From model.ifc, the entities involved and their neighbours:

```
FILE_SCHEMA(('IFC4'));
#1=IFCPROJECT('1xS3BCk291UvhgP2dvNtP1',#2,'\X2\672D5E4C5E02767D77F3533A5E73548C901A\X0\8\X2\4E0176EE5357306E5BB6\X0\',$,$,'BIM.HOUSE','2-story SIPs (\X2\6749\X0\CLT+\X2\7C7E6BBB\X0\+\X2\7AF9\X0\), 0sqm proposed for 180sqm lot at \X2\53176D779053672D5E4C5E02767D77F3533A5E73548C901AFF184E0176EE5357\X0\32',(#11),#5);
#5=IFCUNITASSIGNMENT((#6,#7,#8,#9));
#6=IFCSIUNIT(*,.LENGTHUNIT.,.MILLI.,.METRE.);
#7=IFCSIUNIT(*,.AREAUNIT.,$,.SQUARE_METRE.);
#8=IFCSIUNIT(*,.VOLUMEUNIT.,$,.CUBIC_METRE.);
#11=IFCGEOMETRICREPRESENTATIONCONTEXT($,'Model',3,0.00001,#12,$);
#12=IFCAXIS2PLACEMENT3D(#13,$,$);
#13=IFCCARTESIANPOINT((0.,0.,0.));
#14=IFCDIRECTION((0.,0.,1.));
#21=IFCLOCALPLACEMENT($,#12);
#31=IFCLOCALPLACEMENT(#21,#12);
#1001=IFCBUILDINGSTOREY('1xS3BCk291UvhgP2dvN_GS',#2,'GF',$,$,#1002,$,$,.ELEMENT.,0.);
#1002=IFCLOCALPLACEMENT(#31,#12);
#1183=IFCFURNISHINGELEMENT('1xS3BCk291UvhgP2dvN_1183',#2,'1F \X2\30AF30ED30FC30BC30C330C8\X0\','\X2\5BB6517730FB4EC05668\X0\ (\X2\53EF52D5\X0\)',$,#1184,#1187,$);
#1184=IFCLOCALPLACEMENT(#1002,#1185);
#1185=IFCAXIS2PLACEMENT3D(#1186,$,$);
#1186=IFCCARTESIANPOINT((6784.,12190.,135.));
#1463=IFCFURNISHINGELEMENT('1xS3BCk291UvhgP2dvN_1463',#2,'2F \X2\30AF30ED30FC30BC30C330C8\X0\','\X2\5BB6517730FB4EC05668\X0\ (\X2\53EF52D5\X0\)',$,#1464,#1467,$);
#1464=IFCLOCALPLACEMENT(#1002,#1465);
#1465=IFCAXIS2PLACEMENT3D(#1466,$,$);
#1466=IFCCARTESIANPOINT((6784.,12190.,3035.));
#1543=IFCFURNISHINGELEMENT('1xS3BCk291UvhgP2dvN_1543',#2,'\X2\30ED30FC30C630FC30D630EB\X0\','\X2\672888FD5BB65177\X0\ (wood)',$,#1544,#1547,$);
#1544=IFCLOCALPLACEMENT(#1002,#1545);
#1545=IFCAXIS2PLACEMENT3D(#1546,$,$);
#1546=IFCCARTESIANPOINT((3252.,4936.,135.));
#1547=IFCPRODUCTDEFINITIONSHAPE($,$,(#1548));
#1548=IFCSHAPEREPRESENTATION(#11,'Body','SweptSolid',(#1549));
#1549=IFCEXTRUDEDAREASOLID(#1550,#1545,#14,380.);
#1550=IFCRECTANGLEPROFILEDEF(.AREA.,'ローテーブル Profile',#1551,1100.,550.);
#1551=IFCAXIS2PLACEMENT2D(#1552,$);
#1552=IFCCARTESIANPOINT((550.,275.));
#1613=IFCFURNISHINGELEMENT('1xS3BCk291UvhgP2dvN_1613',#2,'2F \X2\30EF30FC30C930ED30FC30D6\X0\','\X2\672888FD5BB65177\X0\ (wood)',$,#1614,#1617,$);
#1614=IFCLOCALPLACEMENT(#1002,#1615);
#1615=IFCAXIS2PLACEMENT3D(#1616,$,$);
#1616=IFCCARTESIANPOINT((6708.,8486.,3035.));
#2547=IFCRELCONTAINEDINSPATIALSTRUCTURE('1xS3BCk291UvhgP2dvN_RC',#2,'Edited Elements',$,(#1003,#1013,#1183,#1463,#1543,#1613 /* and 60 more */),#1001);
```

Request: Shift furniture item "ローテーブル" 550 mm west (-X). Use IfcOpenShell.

```python
import ifcopenshell
import ifcopenshell.api.geometry
import ifcopenshell.util.placement
import ifcopenshell.util.unit

model = ifcopenshell.open("model.ifc")
unit_scale = ifcopenshell.util.unit.calculate_unit_scale(model)

item = model.by_guid("1xS3BCk291UvhgP2dvN_1543")
matrix = ifcopenshell.util.placement.get_local_placement(item.ObjectPlacement)
matrix[0, 3] -= 0.55 / unit_scale
ifcopenshell.api.geometry.edit_object_placement(model, product=item, matrix=matrix, is_si=False)

print(ifcopenshell.util.placement.get_local_placement(item.ObjectPlacement).round(3) + 0.0)

model.write("model_v2.ifc")
```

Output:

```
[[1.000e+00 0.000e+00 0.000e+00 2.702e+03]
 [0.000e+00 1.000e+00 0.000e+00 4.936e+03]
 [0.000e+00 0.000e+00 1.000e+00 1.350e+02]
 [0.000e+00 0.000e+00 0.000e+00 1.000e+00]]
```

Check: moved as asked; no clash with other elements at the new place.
